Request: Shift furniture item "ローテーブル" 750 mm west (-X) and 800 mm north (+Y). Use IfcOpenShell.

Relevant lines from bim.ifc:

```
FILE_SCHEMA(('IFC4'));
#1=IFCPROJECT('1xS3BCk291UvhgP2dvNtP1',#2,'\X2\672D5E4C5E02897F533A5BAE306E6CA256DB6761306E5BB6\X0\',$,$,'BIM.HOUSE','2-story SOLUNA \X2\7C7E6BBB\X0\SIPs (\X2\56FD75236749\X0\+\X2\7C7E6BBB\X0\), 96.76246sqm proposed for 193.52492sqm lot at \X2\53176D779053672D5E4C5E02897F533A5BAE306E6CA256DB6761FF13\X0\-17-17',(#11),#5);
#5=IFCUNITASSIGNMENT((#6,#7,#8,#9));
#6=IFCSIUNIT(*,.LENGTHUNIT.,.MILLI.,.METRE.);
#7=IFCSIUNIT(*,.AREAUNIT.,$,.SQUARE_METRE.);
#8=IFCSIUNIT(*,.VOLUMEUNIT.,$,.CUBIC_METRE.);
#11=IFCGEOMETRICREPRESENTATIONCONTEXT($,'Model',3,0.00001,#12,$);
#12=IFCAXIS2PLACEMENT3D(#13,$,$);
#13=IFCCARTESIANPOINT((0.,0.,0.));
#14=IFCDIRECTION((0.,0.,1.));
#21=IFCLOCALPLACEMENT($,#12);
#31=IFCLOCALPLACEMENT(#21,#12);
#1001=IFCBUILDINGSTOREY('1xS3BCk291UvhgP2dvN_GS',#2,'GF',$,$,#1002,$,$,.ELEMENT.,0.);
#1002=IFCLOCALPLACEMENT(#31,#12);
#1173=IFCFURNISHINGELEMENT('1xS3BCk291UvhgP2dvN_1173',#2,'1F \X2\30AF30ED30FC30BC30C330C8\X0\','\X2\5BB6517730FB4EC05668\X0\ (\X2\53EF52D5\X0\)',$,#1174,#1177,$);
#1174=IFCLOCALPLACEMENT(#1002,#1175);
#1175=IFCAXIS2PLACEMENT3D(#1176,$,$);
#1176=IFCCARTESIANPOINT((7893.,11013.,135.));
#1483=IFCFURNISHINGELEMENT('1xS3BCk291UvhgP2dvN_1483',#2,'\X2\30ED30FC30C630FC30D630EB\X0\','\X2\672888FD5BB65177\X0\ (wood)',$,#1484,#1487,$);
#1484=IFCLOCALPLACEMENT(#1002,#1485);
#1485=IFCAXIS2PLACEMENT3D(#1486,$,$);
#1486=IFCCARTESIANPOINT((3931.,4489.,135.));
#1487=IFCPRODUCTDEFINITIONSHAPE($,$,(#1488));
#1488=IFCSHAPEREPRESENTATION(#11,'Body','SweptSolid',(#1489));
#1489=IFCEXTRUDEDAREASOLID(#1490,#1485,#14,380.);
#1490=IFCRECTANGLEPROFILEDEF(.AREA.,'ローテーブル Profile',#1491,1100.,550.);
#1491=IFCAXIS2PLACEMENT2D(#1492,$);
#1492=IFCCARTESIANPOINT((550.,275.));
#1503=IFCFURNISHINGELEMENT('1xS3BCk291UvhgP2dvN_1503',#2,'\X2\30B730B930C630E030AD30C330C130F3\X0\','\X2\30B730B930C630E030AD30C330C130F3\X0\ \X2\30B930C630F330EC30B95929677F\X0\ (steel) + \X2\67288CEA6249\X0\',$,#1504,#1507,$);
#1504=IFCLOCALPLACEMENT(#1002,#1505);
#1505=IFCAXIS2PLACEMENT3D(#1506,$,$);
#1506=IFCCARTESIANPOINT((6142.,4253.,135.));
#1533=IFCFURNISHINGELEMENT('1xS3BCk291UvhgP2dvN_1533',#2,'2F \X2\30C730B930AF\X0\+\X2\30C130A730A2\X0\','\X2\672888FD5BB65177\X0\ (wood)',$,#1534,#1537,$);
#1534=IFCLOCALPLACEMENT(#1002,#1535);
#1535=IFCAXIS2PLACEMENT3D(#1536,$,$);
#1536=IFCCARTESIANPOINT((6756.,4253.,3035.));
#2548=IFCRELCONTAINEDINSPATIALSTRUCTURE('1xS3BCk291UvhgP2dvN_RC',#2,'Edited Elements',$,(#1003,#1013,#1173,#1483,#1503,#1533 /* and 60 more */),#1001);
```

```python
import ifcopenshell
import ifcopenshell.api.geometry
import ifcopenshell.util.placement

model = ifcopenshell.open("bim.ifc")

item = model.by_guid("1xS3BCk291UvhgP2dvN_1483")
matrix = ifcopenshell.util.placement.get_local_placement(item.ObjectPlacement)
matrix[0, 3] -= 750.0
matrix[1, 3] += 800.0
ifcopenshell.api.geometry.edit_object_placement(model, product=item, matrix=matrix, is_si=False)

print(ifcopenshell.util.placement.get_local_placement(item.ObjectPlacement).round(3) + 0.0)

model.write("bim_edited.ifc")
```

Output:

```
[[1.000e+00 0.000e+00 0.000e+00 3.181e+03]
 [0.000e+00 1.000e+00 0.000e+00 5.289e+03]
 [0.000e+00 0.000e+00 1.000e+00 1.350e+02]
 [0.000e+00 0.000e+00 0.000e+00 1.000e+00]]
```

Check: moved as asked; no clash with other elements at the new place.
